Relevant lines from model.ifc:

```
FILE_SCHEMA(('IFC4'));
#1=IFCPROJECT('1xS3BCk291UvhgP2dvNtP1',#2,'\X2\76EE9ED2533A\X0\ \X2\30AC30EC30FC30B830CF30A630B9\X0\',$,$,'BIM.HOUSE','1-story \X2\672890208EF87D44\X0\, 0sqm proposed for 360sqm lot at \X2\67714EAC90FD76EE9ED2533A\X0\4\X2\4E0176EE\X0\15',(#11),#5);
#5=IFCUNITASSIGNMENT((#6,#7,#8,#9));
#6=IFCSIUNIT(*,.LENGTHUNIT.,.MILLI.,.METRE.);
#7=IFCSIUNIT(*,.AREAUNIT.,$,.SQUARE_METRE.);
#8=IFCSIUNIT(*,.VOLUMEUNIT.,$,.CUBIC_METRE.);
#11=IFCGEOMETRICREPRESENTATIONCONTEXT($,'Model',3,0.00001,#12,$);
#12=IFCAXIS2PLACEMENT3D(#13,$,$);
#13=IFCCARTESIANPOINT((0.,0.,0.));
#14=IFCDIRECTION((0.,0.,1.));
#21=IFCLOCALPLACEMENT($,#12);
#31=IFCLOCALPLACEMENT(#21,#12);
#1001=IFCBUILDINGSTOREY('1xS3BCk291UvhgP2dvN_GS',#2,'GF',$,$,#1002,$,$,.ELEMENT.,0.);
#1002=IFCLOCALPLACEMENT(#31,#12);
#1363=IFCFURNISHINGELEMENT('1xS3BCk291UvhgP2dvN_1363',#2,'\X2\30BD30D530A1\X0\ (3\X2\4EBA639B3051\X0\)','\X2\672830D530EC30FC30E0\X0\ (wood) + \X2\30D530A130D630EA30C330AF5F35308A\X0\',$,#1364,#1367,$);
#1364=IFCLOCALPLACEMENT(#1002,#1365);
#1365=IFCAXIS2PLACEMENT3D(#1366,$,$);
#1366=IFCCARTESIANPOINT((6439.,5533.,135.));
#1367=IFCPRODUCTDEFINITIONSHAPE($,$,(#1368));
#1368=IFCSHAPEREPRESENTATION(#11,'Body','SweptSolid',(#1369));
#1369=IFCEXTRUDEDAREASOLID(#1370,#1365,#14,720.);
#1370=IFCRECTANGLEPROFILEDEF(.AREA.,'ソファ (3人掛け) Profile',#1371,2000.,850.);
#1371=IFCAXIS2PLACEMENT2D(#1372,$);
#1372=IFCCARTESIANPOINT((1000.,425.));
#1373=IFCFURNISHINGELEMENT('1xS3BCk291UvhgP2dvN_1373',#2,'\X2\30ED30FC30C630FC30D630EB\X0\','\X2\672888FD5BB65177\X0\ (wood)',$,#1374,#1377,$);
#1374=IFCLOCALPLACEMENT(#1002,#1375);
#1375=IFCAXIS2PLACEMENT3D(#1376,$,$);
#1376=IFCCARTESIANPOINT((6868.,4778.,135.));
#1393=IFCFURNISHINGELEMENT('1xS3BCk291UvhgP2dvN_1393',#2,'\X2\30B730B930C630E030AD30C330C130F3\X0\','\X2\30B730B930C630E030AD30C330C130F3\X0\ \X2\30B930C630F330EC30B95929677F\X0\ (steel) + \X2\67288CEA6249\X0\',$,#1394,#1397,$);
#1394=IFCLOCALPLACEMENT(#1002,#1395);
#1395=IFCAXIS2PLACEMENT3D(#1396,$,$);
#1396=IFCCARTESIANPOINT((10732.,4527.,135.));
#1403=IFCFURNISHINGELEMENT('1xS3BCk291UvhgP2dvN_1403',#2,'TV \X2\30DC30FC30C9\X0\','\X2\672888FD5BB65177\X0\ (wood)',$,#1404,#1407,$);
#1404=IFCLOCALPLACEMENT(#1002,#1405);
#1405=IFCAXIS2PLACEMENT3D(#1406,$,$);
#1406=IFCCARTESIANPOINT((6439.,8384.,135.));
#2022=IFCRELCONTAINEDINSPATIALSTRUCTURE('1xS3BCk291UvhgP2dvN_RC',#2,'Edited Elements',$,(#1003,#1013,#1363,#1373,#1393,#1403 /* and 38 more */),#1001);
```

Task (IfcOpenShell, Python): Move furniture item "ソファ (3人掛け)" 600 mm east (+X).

```python
import ifcopenshell
import ifcopenshell.api.geometry
import ifcopenshell.util.placement
import ifcopenshell.util.unit

model = ifcopenshell.open("model.ifc")
unit_scale = ifcopenshell.util.unit.calculate_unit_scale(model)

item = model.by_guid("1xS3BCk291UvhgP2dvN_1363")
matrix = ifcopenshell.util.placement.get_local_placement(item.ObjectPlacement)
matrix[0, 3] += 0.6 / unit_scale
ifcopenshell.api.geometry.edit_object_placement(model, product=item, matrix=matrix, is_si=False)

print(ifcopenshell.util.placement.get_local_placement(item.ObjectPlacement).round(3) + 0.0)

model.write("model_v2.ifc")
```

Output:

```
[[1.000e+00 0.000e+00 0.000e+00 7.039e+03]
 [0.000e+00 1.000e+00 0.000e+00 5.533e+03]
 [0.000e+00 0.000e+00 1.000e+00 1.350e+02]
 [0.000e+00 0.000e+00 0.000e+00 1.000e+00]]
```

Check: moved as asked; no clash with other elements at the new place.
